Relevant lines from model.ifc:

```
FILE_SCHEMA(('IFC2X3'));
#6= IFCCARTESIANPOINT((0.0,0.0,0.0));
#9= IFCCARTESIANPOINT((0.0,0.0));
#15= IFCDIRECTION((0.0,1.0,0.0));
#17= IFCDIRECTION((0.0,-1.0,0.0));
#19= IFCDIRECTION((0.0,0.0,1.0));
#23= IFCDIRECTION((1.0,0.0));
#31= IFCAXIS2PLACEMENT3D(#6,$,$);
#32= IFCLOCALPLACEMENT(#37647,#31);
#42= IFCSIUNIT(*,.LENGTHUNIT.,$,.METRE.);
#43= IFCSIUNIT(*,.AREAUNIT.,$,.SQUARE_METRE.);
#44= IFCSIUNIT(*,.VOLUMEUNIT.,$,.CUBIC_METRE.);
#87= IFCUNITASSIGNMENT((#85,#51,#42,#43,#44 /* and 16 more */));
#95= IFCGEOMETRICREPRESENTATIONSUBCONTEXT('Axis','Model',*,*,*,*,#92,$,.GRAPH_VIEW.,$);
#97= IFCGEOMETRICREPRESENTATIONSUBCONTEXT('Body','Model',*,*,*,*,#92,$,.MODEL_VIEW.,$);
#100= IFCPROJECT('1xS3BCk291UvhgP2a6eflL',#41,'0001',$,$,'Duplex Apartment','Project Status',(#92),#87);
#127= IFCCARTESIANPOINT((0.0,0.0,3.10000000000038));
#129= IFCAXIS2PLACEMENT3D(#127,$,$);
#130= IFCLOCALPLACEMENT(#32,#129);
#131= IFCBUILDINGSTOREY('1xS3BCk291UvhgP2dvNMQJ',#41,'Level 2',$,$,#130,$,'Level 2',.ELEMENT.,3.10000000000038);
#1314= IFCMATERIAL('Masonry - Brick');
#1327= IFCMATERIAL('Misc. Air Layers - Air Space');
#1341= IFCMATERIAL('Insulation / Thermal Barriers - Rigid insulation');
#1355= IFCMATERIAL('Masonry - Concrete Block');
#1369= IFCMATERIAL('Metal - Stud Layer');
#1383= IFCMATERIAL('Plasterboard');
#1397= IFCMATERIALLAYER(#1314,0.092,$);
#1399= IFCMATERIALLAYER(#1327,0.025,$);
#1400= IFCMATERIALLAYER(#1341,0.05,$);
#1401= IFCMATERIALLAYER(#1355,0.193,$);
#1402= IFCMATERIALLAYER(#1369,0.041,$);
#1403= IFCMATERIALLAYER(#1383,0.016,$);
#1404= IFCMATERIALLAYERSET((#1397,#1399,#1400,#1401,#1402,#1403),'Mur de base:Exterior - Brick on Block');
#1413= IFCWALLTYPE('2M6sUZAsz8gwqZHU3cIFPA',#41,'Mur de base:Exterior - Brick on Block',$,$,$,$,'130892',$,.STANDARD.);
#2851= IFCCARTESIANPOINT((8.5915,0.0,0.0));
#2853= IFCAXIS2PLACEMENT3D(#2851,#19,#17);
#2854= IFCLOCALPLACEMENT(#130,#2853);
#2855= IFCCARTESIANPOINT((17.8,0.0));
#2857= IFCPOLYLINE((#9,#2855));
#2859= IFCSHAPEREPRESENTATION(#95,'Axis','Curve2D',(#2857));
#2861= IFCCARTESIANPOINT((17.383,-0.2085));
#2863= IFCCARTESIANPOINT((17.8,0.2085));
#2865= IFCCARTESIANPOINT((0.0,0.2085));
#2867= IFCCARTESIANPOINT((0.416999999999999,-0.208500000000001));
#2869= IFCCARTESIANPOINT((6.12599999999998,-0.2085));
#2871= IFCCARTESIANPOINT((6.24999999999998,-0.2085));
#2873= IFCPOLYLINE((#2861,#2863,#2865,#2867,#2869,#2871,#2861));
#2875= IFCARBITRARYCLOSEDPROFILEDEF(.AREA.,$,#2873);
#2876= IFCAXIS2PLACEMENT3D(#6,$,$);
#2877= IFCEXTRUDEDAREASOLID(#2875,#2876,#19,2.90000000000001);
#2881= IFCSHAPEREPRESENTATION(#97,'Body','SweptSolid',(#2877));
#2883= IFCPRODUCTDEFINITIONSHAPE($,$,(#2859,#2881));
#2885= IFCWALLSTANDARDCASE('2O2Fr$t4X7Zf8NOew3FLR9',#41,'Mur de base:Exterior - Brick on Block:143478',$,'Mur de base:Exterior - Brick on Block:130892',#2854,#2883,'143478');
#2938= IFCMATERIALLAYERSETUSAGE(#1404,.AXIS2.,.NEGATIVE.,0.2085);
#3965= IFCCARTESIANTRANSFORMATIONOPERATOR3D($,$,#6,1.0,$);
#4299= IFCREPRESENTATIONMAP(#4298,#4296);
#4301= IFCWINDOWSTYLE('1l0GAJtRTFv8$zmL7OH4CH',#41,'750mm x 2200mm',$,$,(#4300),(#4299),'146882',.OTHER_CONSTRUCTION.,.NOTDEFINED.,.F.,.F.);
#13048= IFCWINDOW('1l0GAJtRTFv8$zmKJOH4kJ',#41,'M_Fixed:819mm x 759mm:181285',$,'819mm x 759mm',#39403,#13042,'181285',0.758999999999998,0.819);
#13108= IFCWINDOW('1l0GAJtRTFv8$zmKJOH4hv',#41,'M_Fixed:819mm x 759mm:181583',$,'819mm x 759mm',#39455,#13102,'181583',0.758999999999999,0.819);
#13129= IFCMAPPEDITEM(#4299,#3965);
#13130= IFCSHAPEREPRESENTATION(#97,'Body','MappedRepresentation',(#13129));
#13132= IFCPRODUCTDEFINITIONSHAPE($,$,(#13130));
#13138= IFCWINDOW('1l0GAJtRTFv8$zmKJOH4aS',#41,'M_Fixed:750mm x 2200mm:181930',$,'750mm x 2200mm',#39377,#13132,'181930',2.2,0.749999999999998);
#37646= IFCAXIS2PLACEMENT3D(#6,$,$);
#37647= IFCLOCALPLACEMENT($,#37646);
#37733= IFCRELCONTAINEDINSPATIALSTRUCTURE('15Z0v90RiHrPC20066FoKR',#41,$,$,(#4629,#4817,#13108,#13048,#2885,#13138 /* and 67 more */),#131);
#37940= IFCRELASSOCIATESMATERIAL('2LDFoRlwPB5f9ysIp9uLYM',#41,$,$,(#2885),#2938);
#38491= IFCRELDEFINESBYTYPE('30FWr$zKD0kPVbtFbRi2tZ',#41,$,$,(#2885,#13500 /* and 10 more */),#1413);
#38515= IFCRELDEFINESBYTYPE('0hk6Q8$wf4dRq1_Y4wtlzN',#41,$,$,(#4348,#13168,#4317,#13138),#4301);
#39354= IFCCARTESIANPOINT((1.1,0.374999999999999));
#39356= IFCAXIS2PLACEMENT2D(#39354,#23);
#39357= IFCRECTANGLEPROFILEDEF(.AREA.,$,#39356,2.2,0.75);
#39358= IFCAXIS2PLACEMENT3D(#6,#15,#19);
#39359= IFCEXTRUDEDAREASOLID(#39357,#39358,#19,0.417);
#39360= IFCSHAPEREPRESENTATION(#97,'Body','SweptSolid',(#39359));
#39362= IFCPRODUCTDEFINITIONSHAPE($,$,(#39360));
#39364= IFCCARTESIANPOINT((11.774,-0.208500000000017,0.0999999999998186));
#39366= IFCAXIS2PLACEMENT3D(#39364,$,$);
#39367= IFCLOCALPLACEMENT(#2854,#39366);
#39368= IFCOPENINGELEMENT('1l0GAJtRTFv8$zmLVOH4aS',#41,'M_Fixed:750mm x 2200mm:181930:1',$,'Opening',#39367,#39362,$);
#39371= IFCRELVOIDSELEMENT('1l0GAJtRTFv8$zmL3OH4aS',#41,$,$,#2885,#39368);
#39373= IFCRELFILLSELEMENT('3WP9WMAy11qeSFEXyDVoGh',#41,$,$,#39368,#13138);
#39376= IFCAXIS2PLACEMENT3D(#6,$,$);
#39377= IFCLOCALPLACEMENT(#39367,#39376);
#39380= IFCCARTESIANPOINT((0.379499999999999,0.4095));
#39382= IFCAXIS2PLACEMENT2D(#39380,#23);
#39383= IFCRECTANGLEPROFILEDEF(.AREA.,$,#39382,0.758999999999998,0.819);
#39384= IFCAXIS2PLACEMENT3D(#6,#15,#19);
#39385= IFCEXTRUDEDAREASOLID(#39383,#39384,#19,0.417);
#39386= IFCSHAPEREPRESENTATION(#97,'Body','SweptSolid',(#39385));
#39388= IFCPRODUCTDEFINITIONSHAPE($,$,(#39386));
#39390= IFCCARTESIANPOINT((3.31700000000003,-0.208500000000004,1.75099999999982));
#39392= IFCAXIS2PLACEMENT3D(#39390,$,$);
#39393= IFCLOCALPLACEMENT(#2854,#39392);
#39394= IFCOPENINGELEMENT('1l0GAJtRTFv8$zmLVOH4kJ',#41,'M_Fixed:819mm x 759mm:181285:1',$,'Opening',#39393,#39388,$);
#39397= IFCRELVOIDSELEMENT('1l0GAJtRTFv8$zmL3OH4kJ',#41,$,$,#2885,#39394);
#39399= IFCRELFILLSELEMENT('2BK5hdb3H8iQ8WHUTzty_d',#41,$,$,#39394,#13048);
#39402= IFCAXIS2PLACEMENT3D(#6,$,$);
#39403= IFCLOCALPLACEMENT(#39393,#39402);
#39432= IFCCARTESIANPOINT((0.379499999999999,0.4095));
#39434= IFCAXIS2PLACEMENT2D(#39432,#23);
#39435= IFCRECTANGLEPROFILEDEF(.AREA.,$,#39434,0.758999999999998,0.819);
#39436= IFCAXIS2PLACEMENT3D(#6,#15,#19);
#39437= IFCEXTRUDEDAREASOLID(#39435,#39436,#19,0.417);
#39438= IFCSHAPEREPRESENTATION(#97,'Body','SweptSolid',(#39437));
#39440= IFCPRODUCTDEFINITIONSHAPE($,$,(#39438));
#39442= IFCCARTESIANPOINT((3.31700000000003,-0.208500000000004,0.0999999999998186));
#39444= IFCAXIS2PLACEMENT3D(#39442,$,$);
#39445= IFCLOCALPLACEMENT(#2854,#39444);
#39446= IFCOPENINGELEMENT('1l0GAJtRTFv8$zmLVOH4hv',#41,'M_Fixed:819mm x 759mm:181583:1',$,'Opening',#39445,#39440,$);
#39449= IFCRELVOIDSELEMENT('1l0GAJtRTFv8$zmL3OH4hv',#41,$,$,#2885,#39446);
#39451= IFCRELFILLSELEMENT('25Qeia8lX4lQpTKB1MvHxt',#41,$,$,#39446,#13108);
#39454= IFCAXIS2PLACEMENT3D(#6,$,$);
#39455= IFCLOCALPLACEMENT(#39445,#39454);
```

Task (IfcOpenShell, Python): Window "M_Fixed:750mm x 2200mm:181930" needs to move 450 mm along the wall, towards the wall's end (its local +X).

```python
import ifcopenshell
import ifcopenshell.api.geometry
import ifcopenshell.util.placement
import ifcopenshell.util.unit

model = ifcopenshell.open("model.ifc")
unit_scale = ifcopenshell.util.unit.calculate_unit_scale(model)

window = model.by_guid("1l0GAJtRTFv8$zmKJOH4aS")
opening = window.FillsVoids[0].RelatingOpeningElement
wall = opening.VoidsElements[0].RelatingBuildingElement

wall_matrix = ifcopenshell.util.placement.get_local_placement(wall.ObjectPlacement)
shift = wall_matrix[:3, 0] * 0.45 / unit_scale
before = ifcopenshell.util.placement.get_local_placement(window.ObjectPlacement)[:3, 3].copy()

# The window is placed relative to its opening, so it follows when the opening moves.
matrix = ifcopenshell.util.placement.get_local_placement(opening.ObjectPlacement)
matrix[:3, 3] += shift
ifcopenshell.api.geometry.edit_object_placement(
    model, product=opening, matrix=matrix, is_si=False, should_transform_children=True
)

after = ifcopenshell.util.placement.get_local_placement(window.ObjectPlacement)[:3, 3]
print("window moved by", (after - before).round(3) + 0.0)

model.write("model_updated.ifc")
```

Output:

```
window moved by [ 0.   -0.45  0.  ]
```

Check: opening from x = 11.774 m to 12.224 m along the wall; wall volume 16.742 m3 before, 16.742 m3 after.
